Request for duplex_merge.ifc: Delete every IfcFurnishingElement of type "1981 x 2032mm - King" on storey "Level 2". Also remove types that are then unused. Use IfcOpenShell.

First a look at what the model holds.

```python
import ifcopenshell
import ifcopenshell.util.element

model = ifcopenshell.open("duplex_merge.ifc")
print(model.schema)
storey = next(s for s in model.by_type("IfcBuildingStorey") if s.Name == "Level 2")
furniture = [e for e in ifcopenshell.util.element.get_decomposition(storey) if e.is_a("IfcFurnishingElement")]
seen = {}
for e in furniture:
    element_type = ifcopenshell.util.element.get_type(e)
    name = element_type.Name if element_type not in (None, e) else None
    seen[name] = seen.get(name, 0) + 1
for name, count in sorted(seen.items(), key=str):
    print(count, "x", name)
```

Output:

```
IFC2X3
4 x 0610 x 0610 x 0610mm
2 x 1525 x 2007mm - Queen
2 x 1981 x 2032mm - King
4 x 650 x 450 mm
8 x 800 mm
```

```python
import ifcopenshell
import ifcopenshell.api.root
import ifcopenshell.util.element

model = ifcopenshell.open("duplex_merge.ifc")

storey = next(s for s in model.by_type("IfcBuildingStorey") if s.Name == "Level 2")
furniture = [e for e in ifcopenshell.util.element.get_decomposition(storey) if e.is_a("IfcFurnishingElement")]
targets = [e for e in furniture if (t := ifcopenshell.util.element.get_type(e)) not in (None, e) and t.Name == "1981 x 2032mm - King"]
types = {ifcopenshell.util.element.get_type(e) for e in targets} - {None, *targets}

for e in targets:
    ifcopenshell.api.root.remove_product(model, product=e)
print(len(targets), "removed")

unused = [t for t in types if not ifcopenshell.util.element.get_types(t)]
for t in unused:
    ifcopenshell.api.root.remove_product(model, product=t)
print(len(unused), "unused types removed")

model.write("duplex_merge_updated.ifc")
```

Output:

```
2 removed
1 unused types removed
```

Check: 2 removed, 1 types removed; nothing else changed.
